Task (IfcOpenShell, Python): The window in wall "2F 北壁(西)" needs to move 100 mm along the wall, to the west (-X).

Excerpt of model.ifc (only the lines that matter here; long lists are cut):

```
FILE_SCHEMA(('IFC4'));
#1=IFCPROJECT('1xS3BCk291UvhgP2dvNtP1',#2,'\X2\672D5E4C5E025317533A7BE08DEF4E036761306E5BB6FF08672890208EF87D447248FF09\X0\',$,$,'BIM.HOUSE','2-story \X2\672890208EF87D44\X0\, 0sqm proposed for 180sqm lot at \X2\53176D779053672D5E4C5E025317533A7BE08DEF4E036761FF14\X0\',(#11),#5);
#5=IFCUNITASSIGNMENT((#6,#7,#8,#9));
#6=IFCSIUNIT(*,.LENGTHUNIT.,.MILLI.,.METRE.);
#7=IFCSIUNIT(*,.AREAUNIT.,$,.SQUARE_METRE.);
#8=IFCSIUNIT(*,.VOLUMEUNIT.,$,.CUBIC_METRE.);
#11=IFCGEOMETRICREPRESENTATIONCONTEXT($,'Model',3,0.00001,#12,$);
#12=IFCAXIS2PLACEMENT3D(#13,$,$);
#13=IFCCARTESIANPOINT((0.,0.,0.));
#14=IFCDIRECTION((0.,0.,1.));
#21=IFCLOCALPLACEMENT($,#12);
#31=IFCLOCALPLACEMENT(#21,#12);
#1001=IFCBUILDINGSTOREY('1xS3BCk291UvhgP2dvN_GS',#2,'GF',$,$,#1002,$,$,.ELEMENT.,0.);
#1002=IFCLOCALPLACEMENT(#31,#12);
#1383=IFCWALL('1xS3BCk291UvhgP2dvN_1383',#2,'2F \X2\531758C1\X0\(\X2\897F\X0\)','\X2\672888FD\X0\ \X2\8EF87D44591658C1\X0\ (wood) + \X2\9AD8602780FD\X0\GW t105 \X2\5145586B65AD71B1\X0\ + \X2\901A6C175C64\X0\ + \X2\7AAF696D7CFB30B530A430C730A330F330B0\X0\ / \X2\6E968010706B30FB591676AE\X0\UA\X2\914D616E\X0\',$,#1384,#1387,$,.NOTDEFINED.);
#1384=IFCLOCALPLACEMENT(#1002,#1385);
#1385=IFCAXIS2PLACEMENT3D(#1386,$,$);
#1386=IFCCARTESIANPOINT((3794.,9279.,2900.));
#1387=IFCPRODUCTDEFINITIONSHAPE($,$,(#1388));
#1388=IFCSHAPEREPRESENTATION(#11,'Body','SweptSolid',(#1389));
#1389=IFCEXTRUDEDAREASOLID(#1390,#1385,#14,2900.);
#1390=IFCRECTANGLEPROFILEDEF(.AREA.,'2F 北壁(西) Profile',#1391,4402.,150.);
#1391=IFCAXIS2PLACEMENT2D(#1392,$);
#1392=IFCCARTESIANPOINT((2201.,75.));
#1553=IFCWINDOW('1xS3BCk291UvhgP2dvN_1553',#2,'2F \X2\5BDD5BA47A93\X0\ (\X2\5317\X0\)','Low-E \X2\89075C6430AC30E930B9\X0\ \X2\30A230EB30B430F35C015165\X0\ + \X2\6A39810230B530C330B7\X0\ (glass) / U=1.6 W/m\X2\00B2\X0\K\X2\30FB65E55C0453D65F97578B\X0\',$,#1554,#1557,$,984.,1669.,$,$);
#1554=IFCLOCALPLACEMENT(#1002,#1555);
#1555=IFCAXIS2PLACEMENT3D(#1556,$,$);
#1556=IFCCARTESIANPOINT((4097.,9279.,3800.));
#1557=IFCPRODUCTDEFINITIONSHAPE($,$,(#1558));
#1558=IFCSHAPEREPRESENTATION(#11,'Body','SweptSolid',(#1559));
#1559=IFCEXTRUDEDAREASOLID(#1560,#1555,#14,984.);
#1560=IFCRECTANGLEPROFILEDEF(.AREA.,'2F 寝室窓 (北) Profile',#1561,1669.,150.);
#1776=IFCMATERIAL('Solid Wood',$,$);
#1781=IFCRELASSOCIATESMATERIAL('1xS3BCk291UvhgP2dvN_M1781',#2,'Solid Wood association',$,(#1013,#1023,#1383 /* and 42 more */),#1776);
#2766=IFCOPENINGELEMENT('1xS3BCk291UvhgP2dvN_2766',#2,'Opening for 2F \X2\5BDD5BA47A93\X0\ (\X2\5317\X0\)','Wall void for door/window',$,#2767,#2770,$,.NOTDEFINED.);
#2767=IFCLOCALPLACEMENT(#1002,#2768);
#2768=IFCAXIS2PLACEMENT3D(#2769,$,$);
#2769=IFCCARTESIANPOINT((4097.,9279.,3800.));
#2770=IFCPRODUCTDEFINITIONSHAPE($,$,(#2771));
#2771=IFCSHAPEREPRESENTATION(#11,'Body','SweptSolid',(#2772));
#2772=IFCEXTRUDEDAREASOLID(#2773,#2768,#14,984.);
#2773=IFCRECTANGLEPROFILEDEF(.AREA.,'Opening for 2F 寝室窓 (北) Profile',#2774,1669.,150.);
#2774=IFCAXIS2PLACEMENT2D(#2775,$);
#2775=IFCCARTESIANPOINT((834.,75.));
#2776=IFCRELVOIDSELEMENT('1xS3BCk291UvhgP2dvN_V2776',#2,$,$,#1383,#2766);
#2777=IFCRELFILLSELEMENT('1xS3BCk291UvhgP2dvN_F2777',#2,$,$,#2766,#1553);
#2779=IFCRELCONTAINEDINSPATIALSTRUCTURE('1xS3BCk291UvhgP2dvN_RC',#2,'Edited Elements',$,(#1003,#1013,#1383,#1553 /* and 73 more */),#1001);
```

```python
import ifcopenshell
import ifcopenshell.api.geometry
import ifcopenshell.util.placement

model = ifcopenshell.open("model.ifc")

window = model.by_guid("1xS3BCk291UvhgP2dvN_1553")
opening = window.FillsVoids[0].RelatingOpeningElement
wall = opening.VoidsElements[0].RelatingBuildingElement

wall_matrix = ifcopenshell.util.placement.get_local_placement(wall.ObjectPlacement)
shift = wall_matrix[:3, 0] * -100.0
before = ifcopenshell.util.placement.get_local_placement(window.ObjectPlacement)[:3, 3].copy()

# The window is not placed relative to its opening, so move both.
for product in (opening, window):
    matrix = ifcopenshell.util.placement.get_local_placement(product.ObjectPlacement)
    matrix[:3, 3] += shift
    ifcopenshell.api.geometry.edit_object_placement(model, product=product, matrix=matrix, is_si=False)

after = ifcopenshell.util.placement.get_local_placement(window.ObjectPlacement)[:3, 3]
print("window moved by", (after - before).round(3) + 0.0)

model.write("model-out.ifc")
```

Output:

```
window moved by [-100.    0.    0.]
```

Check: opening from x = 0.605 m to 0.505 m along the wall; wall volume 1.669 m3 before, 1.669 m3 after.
